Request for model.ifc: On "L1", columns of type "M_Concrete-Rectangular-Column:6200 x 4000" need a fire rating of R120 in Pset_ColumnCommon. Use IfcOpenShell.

First a look at what the model holds.

```python
import ifcopenshell
import ifcopenshell.util.element

model = ifcopenshell.open("model.ifc")
print(model.schema)
storey = next(s for s in model.by_type("IfcBuildingStorey") if s.Name == "L1")
columns = [e for e in ifcopenshell.util.element.get_decomposition(storey) if e.is_a("IfcColumn")]
seen = {}
for e in columns:
    element_type = ifcopenshell.util.element.get_type(e)
    key = (element_type.Name if element_type != e and element_type else None, ifcopenshell.util.element.get_pset(e, "Pset_ColumnCommon", "FireRating"))
    seen[key] = seen.get(key, 0) + 1
for (name, value), count in sorted(seen.items(), key=str):
    print(count, "x", name, "|", value)
```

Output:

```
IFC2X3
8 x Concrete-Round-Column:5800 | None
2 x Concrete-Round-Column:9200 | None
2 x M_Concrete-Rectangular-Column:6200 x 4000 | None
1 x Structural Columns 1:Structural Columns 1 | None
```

```python
import ifcopenshell
import ifcopenshell.api.pset
import ifcopenshell.util.element

model = ifcopenshell.open("model.ifc")

storey = next(s for s in model.by_type("IfcBuildingStorey") if s.Name == "L1")
columns = [e for e in ifcopenshell.util.element.get_decomposition(storey) if e.is_a("IfcColumn")]

count = 0
for e in columns:
    element_type = ifcopenshell.util.element.get_type(e)
    if element_type in (None, e) or element_type.Name != "M_Concrete-Rectangular-Column:6200 x 4000":
        continue
    # add_pset returns the element's existing set when there is one.
    pset = ifcopenshell.api.pset.add_pset(model, product=e, name="Pset_ColumnCommon")
    ifcopenshell.api.pset.edit_pset(model, pset=pset, properties={"FireRating": "R120"})
    count += 1

print(count, "columns updated")

model.write("model_edited.ifc")
```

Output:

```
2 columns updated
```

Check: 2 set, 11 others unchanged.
